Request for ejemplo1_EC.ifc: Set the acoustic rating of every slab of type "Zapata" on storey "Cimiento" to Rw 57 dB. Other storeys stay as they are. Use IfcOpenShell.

First a look at what the model holds.

```python
import ifcopenshell
import ifcopenshell.util.element

model = ifcopenshell.open("ejemplo1_EC.ifc")
print(model.schema)
storey = next(s for s in model.by_type("IfcBuildingStorey") if s.Name == "Cimiento")
slabs = [e for e in ifcopenshell.util.element.get_decomposition(storey) if e.is_a("IfcSlab")]
seen = {}
for e in slabs:
    element_type = ifcopenshell.util.element.get_type(e)
    key = (element_type.Name if element_type != e and element_type else None, ifcopenshell.util.element.get_pset(e, "Pset_SlabCommon", "AcousticRating"))
    seen[key] = seen.get(key, 0) + 1
for (name, value), count in sorted(seen.items(), key=str):
    print(count, "x", name, "|", value)
```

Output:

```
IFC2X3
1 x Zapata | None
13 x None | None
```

```python
import ifcopenshell
import ifcopenshell.api.pset
import ifcopenshell.util.element

model = ifcopenshell.open("ejemplo1_EC.ifc")

storey = next(s for s in model.by_type("IfcBuildingStorey") if s.Name == "Cimiento")
slabs = [e for e in ifcopenshell.util.element.get_decomposition(storey) if e.is_a("IfcSlab")]

count = 0
for e in slabs:
    element_type = ifcopenshell.util.element.get_type(e)
    if element_type in (None, e) or element_type.Name != "Zapata":
        continue
    # add_pset returns the element's existing set when there is one.
    pset = ifcopenshell.api.pset.add_pset(model, product=e, name="Pset_SlabCommon")
    ifcopenshell.api.pset.edit_pset(model, pset=pset, properties={"AcousticRating": "Rw 57 dB"})
    count += 1

print(count, "slabs updated")

model.write("ejemplo1_EC_v2.ifc")
```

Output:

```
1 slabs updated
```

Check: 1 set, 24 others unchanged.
